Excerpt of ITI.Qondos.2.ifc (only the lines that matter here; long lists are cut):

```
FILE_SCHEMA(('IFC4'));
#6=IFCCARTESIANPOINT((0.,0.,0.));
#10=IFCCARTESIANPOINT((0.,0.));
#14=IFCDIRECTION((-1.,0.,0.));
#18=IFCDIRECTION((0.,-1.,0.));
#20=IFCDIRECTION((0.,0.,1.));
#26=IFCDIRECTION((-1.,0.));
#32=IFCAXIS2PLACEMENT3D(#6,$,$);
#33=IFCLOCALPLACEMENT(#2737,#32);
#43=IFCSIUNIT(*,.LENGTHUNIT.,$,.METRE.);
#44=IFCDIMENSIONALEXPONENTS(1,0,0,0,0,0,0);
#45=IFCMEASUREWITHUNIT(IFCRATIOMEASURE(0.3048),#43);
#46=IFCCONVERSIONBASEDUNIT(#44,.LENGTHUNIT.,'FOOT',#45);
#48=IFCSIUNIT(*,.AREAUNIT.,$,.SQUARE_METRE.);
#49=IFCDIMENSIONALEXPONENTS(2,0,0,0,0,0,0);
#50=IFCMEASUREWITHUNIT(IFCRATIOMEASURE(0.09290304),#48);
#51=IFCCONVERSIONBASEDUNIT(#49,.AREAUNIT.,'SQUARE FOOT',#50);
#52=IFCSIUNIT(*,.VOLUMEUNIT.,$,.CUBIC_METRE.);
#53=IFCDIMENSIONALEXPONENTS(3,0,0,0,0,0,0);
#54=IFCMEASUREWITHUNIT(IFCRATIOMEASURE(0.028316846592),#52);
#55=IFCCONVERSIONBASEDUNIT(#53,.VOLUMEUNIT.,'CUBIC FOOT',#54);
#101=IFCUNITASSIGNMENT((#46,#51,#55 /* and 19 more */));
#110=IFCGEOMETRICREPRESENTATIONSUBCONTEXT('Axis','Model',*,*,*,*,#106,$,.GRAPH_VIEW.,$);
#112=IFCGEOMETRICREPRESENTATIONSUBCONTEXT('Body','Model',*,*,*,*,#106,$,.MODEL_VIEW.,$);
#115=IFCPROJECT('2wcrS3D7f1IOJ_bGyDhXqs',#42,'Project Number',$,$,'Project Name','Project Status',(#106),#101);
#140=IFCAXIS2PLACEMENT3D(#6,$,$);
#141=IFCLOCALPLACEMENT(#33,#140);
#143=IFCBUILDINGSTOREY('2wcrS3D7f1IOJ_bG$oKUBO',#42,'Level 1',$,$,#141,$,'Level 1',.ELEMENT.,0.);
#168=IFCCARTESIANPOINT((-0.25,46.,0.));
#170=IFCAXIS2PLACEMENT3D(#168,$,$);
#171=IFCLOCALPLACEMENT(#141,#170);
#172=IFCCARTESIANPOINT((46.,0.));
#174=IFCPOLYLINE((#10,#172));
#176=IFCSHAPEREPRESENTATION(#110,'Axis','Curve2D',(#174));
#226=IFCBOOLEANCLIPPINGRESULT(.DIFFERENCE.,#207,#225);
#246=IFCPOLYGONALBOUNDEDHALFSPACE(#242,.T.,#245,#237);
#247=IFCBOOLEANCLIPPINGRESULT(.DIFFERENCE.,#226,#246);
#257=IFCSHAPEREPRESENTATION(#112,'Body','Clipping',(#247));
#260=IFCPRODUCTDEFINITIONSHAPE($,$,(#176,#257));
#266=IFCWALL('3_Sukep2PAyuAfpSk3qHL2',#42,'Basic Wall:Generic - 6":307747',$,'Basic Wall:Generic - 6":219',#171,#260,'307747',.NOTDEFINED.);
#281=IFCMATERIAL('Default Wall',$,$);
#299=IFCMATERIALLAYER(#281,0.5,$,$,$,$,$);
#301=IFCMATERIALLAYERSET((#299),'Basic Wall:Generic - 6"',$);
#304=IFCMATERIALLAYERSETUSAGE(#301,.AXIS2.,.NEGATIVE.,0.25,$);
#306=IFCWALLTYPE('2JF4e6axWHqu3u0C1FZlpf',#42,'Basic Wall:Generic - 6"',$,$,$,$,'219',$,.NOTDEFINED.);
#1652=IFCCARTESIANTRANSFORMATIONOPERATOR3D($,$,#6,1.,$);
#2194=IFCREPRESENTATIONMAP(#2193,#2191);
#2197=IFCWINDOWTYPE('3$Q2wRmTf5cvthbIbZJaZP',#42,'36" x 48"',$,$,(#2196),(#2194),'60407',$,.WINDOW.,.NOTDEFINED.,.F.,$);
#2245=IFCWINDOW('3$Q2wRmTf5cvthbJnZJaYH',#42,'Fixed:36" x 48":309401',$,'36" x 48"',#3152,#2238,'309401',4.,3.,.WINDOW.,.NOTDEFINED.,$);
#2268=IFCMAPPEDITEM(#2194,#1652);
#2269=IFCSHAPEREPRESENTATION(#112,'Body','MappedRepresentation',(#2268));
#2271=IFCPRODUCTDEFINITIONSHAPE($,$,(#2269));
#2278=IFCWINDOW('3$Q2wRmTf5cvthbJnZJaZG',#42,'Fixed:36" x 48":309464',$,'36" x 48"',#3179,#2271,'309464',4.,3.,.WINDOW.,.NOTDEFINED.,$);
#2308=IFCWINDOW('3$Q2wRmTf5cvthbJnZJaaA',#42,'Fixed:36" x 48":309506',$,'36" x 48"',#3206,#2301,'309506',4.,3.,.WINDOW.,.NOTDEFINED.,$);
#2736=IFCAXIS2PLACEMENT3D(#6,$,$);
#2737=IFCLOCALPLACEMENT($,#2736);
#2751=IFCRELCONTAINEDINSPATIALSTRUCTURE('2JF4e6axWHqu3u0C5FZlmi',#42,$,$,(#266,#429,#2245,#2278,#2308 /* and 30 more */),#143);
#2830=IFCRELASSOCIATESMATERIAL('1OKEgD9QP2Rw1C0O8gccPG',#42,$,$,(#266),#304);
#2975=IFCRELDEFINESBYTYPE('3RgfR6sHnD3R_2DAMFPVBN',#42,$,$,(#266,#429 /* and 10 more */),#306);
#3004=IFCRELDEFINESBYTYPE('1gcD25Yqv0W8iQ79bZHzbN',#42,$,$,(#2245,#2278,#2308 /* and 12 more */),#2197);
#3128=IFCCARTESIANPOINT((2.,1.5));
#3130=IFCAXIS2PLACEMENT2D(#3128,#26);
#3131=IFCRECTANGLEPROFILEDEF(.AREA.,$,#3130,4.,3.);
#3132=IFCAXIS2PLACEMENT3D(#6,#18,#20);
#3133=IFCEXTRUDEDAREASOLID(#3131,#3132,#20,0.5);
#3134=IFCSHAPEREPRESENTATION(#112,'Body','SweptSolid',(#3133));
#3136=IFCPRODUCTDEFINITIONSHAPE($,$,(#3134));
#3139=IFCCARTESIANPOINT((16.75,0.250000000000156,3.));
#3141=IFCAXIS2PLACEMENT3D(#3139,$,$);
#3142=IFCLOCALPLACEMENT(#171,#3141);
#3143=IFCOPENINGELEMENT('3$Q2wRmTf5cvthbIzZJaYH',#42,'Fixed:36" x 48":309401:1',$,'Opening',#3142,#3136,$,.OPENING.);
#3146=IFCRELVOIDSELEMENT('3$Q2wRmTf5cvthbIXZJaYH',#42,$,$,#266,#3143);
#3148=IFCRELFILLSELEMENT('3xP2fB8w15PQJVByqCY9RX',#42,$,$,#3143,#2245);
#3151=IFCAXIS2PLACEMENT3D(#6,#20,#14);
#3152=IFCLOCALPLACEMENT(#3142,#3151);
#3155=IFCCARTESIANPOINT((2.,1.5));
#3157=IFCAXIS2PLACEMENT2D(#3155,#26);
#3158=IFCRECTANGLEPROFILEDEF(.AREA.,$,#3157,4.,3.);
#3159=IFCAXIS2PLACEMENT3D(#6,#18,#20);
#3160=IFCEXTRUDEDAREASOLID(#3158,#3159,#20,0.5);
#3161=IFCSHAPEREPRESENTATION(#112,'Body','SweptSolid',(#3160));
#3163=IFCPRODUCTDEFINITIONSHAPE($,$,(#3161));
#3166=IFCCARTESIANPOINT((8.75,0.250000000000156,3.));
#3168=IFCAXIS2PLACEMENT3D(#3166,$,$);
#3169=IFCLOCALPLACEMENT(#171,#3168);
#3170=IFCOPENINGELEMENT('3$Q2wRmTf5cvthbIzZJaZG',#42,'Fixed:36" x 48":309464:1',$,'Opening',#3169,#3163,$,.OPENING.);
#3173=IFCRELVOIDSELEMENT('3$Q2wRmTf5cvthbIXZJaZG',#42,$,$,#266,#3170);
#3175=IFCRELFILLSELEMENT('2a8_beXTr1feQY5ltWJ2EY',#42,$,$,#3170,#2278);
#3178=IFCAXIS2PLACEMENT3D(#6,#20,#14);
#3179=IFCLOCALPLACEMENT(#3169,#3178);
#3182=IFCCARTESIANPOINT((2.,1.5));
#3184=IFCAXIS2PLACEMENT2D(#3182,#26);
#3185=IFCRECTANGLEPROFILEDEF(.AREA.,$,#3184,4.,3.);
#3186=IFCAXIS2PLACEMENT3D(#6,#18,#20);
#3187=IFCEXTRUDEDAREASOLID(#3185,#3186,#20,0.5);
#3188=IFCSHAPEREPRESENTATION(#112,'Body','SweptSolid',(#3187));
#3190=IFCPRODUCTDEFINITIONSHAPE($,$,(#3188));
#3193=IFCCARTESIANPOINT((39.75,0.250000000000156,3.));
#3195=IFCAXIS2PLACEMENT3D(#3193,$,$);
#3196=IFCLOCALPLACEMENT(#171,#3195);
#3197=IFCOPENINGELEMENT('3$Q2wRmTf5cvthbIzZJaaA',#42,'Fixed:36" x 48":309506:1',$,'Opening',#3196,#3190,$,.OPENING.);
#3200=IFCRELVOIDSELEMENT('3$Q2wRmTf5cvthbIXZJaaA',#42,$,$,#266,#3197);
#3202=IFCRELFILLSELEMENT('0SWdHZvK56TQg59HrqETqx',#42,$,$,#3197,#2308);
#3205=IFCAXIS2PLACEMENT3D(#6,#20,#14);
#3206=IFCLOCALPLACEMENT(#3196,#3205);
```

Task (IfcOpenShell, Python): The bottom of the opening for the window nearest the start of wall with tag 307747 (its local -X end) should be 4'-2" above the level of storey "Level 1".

```python
import numpy as np
import ifcopenshell
import ifcopenshell.api.geometry
import ifcopenshell.geom
import ifcopenshell.util.element
import ifcopenshell.util.placement
import ifcopenshell.util.shape
import ifcopenshell.util.unit

model = ifcopenshell.open("ITI.Qondos.2.ifc")
unit_scale = ifcopenshell.util.unit.calculate_unit_scale(model)

window = model.by_guid("3$Q2wRmTf5cvthbJnZJaZG")
opening = window.FillsVoids[0].RelatingOpeningElement
storey = ifcopenshell.util.element.get_container(window, ifc_class="IfcBuildingStorey")
level = ifcopenshell.util.placement.get_local_placement(storey.ObjectPlacement)[2, 3]

# The opening's origin need not be at the sill, so measure its lowest point.
shape = ifcopenshell.geom.create_shape(ifcopenshell.geom.settings(), opening)
bottom = ifcopenshell.util.shape.get_shape_bottom_elevation(shape, shape.geometry) / unit_scale
dz = level + 50 * 0.0254 / unit_scale - bottom

shift = np.array([0.0, 0.0, dz])
# The window is placed relative to its opening, so it follows when the opening moves.
matrix = ifcopenshell.util.placement.get_local_placement(opening.ObjectPlacement)
matrix[:3, 3] += shift
ifcopenshell.api.geometry.edit_object_placement(
    model, product=opening, matrix=matrix, is_si=False, should_transform_children=True
)

print(f"moved by {dz * unit_scale:+.3f} m")

model.write("ITI.Qondos.2_updated.ifc")
```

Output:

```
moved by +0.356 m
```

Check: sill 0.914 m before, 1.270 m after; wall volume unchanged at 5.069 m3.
